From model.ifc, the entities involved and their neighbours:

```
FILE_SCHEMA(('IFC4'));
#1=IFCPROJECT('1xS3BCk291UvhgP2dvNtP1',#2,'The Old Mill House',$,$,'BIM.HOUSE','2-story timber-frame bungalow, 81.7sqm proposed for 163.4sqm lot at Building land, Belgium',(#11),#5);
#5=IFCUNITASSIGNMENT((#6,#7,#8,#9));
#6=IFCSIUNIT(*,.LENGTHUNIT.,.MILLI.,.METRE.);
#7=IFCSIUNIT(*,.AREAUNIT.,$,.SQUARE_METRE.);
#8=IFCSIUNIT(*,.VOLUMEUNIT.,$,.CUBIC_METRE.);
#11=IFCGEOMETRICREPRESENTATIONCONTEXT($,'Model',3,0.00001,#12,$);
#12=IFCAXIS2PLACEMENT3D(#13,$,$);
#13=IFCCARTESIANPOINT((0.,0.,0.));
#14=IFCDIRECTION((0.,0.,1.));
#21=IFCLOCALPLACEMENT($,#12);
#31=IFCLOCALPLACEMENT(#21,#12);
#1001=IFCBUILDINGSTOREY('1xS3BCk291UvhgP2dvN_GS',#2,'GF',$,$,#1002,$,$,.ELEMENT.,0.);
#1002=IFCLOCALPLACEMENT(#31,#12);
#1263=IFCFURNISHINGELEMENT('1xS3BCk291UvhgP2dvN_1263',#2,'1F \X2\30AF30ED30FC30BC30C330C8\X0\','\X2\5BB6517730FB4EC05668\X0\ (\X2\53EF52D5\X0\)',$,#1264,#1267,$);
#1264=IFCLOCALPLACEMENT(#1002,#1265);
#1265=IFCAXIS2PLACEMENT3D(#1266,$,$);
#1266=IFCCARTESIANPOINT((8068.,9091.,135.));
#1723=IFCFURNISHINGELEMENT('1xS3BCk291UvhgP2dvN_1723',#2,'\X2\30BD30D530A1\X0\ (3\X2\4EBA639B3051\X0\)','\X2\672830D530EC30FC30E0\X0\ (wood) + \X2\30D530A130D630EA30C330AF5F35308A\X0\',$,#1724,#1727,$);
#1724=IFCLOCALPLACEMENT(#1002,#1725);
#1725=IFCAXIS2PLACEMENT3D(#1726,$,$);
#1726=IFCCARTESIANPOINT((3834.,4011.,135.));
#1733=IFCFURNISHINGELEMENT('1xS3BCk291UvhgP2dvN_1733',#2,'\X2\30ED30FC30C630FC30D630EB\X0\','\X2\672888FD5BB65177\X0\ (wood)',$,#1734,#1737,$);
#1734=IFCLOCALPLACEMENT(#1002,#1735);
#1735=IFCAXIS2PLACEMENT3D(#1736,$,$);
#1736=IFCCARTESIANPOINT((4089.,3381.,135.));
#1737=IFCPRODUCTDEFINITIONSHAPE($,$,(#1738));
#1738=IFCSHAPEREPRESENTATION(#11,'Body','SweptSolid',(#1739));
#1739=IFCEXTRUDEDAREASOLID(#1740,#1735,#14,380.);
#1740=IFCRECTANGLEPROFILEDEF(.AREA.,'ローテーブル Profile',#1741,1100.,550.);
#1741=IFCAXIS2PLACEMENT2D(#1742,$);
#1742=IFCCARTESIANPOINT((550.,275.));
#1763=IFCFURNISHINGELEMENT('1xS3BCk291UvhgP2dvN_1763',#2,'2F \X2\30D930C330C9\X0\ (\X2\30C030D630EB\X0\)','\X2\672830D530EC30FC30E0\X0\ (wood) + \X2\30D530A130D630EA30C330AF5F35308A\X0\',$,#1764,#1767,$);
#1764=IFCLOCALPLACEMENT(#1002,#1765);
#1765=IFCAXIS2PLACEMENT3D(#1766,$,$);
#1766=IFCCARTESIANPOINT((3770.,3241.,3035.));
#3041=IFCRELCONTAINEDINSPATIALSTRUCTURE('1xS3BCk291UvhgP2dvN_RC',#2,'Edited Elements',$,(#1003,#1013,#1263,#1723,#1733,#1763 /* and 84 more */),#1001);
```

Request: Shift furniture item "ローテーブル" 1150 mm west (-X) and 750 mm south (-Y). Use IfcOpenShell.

```python
import ifcopenshell
import ifcopenshell.api.geometry
import ifcopenshell.util.placement
import ifcopenshell.util.unit

model = ifcopenshell.open("model.ifc")
unit_scale = ifcopenshell.util.unit.calculate_unit_scale(model)

item = model.by_guid("1xS3BCk291UvhgP2dvN_1733")
matrix = ifcopenshell.util.placement.get_local_placement(item.ObjectPlacement)
matrix[0, 3] -= 1.15 / unit_scale
matrix[1, 3] -= 0.75 / unit_scale
ifcopenshell.api.geometry.edit_object_placement(model, product=item, matrix=matrix, is_si=False)

print(ifcopenshell.util.placement.get_local_placement(item.ObjectPlacement).round(3) + 0.0)

model.write("model_v2.ifc")
```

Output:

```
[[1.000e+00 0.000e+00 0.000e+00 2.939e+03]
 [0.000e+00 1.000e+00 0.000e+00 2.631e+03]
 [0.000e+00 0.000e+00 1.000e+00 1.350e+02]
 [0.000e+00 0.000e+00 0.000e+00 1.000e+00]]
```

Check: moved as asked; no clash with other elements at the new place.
